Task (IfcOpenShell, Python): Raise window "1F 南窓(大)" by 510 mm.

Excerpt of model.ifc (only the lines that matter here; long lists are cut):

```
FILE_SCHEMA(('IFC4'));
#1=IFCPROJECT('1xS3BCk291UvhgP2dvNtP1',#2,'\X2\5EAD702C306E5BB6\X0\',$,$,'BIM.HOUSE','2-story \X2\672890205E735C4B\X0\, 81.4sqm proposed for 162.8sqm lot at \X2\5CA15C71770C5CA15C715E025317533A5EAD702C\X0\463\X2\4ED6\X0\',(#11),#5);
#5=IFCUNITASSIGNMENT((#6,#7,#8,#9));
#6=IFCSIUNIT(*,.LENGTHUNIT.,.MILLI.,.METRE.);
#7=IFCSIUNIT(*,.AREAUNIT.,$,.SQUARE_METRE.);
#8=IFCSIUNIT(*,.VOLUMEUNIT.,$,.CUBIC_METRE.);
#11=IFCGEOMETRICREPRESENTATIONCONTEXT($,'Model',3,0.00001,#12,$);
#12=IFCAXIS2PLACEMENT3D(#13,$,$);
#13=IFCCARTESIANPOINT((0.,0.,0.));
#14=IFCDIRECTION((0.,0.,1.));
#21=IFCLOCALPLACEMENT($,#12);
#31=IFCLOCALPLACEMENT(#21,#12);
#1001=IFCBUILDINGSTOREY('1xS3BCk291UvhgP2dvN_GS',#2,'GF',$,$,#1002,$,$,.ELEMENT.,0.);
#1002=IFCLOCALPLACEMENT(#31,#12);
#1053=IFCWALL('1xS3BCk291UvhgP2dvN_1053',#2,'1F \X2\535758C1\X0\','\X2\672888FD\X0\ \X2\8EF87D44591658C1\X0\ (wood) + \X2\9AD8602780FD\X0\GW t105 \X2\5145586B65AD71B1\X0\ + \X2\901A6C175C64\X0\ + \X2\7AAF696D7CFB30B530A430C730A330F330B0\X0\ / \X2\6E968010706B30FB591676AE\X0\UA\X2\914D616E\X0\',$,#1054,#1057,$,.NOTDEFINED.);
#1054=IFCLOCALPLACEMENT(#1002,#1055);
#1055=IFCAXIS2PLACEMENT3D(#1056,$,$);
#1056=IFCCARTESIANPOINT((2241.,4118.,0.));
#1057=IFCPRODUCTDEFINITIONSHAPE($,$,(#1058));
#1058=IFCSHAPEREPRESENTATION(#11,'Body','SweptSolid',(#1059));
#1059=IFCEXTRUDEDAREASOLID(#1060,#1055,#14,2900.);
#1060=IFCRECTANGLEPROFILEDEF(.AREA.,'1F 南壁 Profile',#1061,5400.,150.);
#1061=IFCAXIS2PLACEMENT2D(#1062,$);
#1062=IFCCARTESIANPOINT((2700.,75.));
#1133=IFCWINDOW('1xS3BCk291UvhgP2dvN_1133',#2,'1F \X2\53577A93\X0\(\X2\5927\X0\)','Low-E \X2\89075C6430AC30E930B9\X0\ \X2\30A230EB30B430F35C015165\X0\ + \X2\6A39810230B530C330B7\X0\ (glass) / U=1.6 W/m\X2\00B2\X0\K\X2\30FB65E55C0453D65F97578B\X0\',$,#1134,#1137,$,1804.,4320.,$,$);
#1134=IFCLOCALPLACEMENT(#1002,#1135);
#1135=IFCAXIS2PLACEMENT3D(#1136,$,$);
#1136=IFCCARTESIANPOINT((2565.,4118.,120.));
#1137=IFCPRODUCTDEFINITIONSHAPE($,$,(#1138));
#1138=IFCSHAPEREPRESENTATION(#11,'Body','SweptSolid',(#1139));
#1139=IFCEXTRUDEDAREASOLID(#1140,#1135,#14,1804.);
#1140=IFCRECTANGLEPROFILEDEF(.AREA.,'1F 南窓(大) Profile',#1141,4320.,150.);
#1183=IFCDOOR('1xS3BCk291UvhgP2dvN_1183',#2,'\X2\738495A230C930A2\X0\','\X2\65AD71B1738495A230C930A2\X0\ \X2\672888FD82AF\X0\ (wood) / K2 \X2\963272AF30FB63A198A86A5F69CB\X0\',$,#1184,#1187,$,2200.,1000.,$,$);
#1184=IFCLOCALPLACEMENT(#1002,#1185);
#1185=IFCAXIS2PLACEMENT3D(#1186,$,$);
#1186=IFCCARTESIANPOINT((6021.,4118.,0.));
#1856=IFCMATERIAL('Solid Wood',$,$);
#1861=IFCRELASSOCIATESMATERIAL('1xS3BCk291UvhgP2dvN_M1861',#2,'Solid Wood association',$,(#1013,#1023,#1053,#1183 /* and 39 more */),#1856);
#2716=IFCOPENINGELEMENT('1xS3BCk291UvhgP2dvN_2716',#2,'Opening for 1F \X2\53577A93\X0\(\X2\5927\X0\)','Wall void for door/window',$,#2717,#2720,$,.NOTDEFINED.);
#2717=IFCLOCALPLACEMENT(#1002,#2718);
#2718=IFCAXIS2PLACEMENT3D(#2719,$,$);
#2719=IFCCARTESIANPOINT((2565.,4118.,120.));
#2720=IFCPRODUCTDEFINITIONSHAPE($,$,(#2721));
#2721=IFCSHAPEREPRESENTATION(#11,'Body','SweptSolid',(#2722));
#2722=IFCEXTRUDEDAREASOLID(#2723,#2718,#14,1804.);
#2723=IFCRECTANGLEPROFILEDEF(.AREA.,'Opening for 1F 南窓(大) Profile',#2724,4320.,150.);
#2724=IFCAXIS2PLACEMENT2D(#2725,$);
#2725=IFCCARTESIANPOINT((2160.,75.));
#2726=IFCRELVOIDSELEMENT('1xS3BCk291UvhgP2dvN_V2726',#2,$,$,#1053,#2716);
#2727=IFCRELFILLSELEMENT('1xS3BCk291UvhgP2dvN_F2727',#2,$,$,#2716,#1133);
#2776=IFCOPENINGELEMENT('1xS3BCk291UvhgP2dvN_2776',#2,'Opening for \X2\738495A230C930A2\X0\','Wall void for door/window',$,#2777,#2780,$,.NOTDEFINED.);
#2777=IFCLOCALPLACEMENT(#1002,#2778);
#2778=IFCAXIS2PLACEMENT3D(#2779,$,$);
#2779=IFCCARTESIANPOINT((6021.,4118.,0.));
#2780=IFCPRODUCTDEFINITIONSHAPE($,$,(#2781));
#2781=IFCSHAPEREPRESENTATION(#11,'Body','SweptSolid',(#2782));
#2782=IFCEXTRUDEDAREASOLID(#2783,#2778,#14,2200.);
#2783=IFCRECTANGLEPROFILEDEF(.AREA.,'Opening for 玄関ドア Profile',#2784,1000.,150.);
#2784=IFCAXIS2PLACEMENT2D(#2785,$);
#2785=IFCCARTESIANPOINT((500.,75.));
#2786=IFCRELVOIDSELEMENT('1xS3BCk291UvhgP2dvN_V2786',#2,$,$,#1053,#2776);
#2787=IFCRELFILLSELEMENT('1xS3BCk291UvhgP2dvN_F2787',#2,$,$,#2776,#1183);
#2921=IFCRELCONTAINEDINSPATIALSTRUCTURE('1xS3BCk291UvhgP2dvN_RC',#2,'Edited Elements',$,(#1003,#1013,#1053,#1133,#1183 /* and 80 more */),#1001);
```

```python
import numpy as np
import ifcopenshell
import ifcopenshell.api.geometry
import ifcopenshell.util.placement
import ifcopenshell.util.unit

model = ifcopenshell.open("model.ifc")
unit_scale = ifcopenshell.util.unit.calculate_unit_scale(model)

window = model.by_id(1133)
opening = window.FillsVoids[0].RelatingOpeningElement
dz = 0.51 / unit_scale

shift = np.array([0.0, 0.0, dz])
# The window is not placed relative to its opening, so move both.
for product in (opening, window):
    matrix = ifcopenshell.util.placement.get_local_placement(product.ObjectPlacement)
    matrix[:3, 3] += shift
    ifcopenshell.api.geometry.edit_object_placement(model, product=product, matrix=matrix, is_si=False)

print(f"moved by {dz * unit_scale:+.3f} m")

model.write("model_rev.ifc")
```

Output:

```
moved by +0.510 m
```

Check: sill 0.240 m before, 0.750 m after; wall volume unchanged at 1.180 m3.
